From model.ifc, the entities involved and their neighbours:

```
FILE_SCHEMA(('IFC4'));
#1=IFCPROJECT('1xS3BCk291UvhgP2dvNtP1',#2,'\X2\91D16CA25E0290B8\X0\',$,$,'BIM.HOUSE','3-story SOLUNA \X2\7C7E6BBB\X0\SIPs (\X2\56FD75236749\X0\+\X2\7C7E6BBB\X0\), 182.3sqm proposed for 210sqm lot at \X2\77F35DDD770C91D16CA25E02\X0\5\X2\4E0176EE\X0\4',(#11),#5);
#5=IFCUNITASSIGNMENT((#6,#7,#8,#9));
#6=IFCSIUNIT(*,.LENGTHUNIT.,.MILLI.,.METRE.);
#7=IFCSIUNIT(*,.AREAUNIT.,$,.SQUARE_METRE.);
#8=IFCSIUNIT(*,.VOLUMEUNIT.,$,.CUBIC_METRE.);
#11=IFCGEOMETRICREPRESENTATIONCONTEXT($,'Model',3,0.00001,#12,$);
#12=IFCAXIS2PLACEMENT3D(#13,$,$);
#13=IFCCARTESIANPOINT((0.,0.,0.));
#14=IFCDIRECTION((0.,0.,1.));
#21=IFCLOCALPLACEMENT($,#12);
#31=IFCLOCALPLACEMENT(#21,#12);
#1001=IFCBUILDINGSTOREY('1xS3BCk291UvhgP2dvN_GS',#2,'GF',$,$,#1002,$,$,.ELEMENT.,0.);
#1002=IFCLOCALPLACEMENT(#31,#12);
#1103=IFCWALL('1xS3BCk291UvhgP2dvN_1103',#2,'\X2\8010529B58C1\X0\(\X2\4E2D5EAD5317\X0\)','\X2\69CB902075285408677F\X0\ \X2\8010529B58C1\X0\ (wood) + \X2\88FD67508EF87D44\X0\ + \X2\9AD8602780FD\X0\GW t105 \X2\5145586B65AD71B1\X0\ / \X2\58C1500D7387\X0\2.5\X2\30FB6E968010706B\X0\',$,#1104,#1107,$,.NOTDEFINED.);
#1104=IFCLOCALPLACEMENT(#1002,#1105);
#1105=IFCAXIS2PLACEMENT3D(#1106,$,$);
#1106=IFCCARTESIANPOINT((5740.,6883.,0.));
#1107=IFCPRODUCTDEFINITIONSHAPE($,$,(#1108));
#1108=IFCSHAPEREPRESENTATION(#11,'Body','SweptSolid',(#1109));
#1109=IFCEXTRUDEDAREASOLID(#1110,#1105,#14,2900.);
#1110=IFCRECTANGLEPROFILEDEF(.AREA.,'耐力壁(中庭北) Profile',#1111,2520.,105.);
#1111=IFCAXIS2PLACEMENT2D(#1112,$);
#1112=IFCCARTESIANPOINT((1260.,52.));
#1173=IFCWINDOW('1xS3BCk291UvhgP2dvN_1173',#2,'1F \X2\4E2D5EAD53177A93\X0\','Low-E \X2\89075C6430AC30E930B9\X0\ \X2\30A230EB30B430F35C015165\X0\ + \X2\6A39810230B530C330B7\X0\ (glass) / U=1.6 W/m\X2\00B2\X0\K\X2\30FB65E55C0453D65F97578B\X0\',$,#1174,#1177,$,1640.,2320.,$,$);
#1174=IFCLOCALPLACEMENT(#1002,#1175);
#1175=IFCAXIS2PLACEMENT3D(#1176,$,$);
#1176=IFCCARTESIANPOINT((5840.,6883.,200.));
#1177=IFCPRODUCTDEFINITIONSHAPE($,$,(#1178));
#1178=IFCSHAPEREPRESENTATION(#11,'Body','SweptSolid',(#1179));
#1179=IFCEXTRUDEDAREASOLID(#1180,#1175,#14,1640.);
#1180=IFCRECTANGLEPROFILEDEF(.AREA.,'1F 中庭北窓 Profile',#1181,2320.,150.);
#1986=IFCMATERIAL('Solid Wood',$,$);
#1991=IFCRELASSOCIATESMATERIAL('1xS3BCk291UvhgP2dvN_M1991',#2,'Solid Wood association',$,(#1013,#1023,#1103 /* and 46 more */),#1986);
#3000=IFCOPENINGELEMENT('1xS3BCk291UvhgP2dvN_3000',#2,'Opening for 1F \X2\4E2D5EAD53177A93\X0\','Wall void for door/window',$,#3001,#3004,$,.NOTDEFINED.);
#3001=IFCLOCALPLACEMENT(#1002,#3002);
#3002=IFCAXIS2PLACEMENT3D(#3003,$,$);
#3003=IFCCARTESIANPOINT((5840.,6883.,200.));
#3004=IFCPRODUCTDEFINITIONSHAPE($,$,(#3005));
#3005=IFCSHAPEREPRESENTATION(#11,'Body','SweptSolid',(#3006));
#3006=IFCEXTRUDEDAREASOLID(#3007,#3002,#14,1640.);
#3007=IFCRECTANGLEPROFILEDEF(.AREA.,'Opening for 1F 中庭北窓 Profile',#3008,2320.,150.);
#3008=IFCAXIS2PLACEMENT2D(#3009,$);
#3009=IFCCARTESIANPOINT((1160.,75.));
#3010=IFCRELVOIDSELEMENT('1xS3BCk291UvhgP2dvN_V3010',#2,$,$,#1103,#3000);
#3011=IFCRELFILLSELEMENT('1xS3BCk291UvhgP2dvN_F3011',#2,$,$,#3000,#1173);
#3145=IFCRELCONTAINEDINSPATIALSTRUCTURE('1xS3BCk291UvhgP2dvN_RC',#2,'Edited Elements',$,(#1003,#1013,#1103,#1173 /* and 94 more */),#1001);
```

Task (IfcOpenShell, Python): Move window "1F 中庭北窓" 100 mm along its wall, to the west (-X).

```python
import ifcopenshell
import ifcopenshell.api.geometry
import ifcopenshell.util.placement
import ifcopenshell.util.unit

model = ifcopenshell.open("model.ifc")
unit_scale = ifcopenshell.util.unit.calculate_unit_scale(model)

window = model.by_guid("1xS3BCk291UvhgP2dvN_1173")
opening = window.FillsVoids[0].RelatingOpeningElement
wall = opening.VoidsElements[0].RelatingBuildingElement

wall_matrix = ifcopenshell.util.placement.get_local_placement(wall.ObjectPlacement)
shift = wall_matrix[:3, 0] * -0.1 / unit_scale
before = ifcopenshell.util.placement.get_local_placement(window.ObjectPlacement)[:3, 3].copy()

# The window is not placed relative to its opening, so move both.
for product in (opening, window):
    matrix = ifcopenshell.util.placement.get_local_placement(product.ObjectPlacement)
    matrix[:3, 3] += shift
    ifcopenshell.api.geometry.edit_object_placement(model, product=product, matrix=matrix, is_si=False)

after = ifcopenshell.util.placement.get_local_placement(window.ObjectPlacement)[:3, 3]
print("window moved by", (after - before).round(3) + 0.0)

model.write("model_v2.ifc")
```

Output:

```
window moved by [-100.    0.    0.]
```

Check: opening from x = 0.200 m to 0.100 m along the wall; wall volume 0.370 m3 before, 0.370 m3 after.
